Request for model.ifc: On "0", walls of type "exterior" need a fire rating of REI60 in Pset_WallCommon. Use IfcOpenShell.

First a look at what the model holds.

```python
import ifcopenshell
import ifcopenshell.util.element

model = ifcopenshell.open("model.ifc")
print(model.schema)
storey = next(s for s in model.by_type("IfcBuildingStorey") if s.Name == "0")
walls = [e for e in ifcopenshell.util.element.get_decomposition(storey) if e.is_a("IfcWall")]
seen = {}
for e in walls:
    element_type = ifcopenshell.util.element.get_type(e)
    key = (element_type.Name if element_type != e and element_type else None, ifcopenshell.util.element.get_pset(e, "Pset_WallCommon", "FireRating"))
    seen[key] = seen.get(key, 0) + 1
for (name, value), count in sorted(seen.items(), key=str):
    print(count, "x", name, "|", value)
```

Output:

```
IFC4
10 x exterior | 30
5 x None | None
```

```python
import ifcopenshell
import ifcopenshell.api.pset
import ifcopenshell.util.element

model = ifcopenshell.open("model.ifc")

storey = next(s for s in model.by_type("IfcBuildingStorey") if s.Name == "0")
walls = [e for e in ifcopenshell.util.element.get_decomposition(storey) if e.is_a("IfcWall")]

count = 0
for e in walls:
    element_type = ifcopenshell.util.element.get_type(e)
    if element_type in (None, e) or element_type.Name != "exterior":
        continue
    # add_pset returns the element's existing set when there is one.
    pset = ifcopenshell.api.pset.add_pset(model, product=e, name="Pset_WallCommon")
    ifcopenshell.api.pset.edit_pset(model, pset=pset, properties={"FireRating": "REI60"})
    count += 1

print(count, "walls updated")

model.write("model_updated.ifc")
```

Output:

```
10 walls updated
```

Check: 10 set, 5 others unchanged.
